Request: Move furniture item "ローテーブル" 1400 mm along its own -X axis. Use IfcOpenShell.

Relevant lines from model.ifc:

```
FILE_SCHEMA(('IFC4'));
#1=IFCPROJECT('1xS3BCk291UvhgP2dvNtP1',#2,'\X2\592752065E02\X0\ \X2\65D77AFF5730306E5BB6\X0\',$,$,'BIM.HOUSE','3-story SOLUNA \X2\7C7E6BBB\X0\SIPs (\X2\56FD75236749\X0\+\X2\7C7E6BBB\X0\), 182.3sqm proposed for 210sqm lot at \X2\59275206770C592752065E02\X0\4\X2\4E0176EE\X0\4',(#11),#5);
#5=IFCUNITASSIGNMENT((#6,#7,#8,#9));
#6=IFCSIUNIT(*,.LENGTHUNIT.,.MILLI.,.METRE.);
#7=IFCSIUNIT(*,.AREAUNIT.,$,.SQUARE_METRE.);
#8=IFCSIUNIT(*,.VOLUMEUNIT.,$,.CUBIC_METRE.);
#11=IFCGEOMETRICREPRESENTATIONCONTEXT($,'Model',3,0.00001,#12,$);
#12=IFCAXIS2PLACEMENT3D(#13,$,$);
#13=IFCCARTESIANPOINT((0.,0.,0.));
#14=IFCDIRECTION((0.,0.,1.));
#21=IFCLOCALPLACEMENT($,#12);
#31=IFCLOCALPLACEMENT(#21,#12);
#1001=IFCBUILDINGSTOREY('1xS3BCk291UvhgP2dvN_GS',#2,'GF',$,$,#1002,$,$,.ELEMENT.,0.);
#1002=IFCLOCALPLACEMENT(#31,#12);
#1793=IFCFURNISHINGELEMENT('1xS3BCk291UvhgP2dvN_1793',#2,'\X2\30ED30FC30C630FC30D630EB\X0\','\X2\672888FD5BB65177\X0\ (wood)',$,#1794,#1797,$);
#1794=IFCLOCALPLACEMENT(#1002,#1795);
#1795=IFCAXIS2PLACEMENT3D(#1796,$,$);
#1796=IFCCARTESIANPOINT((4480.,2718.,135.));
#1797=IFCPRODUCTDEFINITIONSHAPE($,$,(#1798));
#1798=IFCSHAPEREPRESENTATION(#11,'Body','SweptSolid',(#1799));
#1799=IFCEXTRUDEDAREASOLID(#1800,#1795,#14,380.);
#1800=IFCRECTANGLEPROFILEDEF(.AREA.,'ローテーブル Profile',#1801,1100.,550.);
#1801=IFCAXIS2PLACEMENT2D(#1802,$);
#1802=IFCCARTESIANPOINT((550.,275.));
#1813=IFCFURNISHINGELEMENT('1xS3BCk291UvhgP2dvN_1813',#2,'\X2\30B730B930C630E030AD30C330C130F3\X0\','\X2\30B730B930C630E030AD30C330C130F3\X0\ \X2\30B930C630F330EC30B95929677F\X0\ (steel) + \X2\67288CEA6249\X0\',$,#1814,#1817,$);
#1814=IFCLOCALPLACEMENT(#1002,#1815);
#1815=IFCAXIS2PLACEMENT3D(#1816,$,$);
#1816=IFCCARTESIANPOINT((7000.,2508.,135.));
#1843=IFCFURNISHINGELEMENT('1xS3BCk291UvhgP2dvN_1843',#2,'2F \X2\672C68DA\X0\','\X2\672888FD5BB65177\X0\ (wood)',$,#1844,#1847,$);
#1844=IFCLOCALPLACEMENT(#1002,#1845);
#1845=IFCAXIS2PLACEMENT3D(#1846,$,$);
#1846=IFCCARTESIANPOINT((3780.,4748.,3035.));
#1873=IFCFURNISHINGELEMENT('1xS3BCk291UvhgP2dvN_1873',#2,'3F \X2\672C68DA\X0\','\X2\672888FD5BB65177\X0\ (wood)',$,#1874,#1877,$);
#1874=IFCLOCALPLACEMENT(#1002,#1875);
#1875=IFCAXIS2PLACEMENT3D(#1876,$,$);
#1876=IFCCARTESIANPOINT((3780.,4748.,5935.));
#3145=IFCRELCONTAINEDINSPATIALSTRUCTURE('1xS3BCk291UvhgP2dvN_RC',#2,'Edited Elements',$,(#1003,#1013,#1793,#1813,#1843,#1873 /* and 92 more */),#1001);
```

```python
import ifcopenshell
import ifcopenshell.api.geometry
import ifcopenshell.util.placement
import ifcopenshell.util.unit

model = ifcopenshell.open("model.ifc")
unit_scale = ifcopenshell.util.unit.calculate_unit_scale(model)

item = model.by_guid("1xS3BCk291UvhgP2dvN_1793")
matrix = ifcopenshell.util.placement.get_local_placement(item.ObjectPlacement)
matrix[:3, 3] -= matrix[:3, 0] * 1.4 / unit_scale
ifcopenshell.api.geometry.edit_object_placement(model, product=item, matrix=matrix, is_si=False)

print(ifcopenshell.util.placement.get_local_placement(item.ObjectPlacement).round(3) + 0.0)

model.write("model_updated.ifc")
```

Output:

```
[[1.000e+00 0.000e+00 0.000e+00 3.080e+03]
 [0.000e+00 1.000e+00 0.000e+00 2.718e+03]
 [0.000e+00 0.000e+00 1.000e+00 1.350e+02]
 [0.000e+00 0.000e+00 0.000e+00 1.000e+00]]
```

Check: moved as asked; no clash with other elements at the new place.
